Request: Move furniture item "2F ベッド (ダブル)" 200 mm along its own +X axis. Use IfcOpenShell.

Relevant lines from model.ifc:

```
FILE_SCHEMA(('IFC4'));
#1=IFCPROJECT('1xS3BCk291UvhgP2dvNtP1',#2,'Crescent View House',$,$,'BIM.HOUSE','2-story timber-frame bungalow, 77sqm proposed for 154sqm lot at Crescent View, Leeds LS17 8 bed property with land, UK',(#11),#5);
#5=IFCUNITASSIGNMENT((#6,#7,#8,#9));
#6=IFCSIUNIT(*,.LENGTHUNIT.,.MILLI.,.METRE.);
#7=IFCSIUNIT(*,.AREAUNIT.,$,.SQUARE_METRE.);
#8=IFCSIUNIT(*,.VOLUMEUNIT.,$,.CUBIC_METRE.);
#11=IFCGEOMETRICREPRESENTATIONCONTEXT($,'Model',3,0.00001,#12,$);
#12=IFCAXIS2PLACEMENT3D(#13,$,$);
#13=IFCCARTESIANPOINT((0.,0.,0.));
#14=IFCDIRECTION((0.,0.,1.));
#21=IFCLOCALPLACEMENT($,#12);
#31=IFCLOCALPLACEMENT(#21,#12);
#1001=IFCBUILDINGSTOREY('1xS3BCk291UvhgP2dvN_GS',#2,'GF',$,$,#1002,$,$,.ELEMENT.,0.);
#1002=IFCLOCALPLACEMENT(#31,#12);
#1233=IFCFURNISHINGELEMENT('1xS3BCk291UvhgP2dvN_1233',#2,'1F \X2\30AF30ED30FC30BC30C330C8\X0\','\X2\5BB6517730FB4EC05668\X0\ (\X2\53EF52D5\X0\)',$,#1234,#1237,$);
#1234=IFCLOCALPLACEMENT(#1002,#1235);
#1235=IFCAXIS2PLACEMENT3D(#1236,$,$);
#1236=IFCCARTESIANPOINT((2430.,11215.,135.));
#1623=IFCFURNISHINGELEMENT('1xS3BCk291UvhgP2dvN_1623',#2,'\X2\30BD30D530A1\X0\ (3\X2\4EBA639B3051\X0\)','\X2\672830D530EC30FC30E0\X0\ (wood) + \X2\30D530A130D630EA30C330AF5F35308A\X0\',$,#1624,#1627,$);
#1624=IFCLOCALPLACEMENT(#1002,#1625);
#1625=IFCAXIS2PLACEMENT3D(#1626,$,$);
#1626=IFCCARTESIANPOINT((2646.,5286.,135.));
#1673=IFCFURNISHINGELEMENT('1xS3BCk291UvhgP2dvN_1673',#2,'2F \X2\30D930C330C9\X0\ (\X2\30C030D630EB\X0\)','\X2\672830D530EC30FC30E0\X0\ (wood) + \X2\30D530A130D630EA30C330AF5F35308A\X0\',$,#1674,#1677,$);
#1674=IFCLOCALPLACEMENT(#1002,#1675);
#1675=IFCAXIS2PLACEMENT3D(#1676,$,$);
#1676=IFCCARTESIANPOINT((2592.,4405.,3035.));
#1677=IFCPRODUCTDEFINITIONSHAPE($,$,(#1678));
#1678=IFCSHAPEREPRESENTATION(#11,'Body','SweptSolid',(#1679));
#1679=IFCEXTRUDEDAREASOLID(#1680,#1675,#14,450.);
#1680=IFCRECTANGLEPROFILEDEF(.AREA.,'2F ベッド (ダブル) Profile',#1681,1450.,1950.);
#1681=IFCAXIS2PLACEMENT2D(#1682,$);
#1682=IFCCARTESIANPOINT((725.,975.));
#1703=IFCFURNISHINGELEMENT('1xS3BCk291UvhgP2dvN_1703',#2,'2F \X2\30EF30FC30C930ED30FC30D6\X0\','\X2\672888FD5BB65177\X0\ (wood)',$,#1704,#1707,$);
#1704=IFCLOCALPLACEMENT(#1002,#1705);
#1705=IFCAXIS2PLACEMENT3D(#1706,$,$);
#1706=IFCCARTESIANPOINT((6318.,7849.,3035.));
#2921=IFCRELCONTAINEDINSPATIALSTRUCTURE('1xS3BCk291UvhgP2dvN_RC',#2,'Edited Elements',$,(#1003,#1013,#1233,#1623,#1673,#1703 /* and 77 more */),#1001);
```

```python
import ifcopenshell
import ifcopenshell.api.geometry
import ifcopenshell.util.placement
import ifcopenshell.util.unit

model = ifcopenshell.open("model.ifc")
unit_scale = ifcopenshell.util.unit.calculate_unit_scale(model)

item = model.by_guid("1xS3BCk291UvhgP2dvN_1673")
matrix = ifcopenshell.util.placement.get_local_placement(item.ObjectPlacement)
matrix[:3, 3] += matrix[:3, 0] * 0.2 / unit_scale
ifcopenshell.api.geometry.edit_object_placement(model, product=item, matrix=matrix, is_si=False)

print(ifcopenshell.util.placement.get_local_placement(item.ObjectPlacement).round(3) + 0.0)

model.write("model_rev.ifc")
```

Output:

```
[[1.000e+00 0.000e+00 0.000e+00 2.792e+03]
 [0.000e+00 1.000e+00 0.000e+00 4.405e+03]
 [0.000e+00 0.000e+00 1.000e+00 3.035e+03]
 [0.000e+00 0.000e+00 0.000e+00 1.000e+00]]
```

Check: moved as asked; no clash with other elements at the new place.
